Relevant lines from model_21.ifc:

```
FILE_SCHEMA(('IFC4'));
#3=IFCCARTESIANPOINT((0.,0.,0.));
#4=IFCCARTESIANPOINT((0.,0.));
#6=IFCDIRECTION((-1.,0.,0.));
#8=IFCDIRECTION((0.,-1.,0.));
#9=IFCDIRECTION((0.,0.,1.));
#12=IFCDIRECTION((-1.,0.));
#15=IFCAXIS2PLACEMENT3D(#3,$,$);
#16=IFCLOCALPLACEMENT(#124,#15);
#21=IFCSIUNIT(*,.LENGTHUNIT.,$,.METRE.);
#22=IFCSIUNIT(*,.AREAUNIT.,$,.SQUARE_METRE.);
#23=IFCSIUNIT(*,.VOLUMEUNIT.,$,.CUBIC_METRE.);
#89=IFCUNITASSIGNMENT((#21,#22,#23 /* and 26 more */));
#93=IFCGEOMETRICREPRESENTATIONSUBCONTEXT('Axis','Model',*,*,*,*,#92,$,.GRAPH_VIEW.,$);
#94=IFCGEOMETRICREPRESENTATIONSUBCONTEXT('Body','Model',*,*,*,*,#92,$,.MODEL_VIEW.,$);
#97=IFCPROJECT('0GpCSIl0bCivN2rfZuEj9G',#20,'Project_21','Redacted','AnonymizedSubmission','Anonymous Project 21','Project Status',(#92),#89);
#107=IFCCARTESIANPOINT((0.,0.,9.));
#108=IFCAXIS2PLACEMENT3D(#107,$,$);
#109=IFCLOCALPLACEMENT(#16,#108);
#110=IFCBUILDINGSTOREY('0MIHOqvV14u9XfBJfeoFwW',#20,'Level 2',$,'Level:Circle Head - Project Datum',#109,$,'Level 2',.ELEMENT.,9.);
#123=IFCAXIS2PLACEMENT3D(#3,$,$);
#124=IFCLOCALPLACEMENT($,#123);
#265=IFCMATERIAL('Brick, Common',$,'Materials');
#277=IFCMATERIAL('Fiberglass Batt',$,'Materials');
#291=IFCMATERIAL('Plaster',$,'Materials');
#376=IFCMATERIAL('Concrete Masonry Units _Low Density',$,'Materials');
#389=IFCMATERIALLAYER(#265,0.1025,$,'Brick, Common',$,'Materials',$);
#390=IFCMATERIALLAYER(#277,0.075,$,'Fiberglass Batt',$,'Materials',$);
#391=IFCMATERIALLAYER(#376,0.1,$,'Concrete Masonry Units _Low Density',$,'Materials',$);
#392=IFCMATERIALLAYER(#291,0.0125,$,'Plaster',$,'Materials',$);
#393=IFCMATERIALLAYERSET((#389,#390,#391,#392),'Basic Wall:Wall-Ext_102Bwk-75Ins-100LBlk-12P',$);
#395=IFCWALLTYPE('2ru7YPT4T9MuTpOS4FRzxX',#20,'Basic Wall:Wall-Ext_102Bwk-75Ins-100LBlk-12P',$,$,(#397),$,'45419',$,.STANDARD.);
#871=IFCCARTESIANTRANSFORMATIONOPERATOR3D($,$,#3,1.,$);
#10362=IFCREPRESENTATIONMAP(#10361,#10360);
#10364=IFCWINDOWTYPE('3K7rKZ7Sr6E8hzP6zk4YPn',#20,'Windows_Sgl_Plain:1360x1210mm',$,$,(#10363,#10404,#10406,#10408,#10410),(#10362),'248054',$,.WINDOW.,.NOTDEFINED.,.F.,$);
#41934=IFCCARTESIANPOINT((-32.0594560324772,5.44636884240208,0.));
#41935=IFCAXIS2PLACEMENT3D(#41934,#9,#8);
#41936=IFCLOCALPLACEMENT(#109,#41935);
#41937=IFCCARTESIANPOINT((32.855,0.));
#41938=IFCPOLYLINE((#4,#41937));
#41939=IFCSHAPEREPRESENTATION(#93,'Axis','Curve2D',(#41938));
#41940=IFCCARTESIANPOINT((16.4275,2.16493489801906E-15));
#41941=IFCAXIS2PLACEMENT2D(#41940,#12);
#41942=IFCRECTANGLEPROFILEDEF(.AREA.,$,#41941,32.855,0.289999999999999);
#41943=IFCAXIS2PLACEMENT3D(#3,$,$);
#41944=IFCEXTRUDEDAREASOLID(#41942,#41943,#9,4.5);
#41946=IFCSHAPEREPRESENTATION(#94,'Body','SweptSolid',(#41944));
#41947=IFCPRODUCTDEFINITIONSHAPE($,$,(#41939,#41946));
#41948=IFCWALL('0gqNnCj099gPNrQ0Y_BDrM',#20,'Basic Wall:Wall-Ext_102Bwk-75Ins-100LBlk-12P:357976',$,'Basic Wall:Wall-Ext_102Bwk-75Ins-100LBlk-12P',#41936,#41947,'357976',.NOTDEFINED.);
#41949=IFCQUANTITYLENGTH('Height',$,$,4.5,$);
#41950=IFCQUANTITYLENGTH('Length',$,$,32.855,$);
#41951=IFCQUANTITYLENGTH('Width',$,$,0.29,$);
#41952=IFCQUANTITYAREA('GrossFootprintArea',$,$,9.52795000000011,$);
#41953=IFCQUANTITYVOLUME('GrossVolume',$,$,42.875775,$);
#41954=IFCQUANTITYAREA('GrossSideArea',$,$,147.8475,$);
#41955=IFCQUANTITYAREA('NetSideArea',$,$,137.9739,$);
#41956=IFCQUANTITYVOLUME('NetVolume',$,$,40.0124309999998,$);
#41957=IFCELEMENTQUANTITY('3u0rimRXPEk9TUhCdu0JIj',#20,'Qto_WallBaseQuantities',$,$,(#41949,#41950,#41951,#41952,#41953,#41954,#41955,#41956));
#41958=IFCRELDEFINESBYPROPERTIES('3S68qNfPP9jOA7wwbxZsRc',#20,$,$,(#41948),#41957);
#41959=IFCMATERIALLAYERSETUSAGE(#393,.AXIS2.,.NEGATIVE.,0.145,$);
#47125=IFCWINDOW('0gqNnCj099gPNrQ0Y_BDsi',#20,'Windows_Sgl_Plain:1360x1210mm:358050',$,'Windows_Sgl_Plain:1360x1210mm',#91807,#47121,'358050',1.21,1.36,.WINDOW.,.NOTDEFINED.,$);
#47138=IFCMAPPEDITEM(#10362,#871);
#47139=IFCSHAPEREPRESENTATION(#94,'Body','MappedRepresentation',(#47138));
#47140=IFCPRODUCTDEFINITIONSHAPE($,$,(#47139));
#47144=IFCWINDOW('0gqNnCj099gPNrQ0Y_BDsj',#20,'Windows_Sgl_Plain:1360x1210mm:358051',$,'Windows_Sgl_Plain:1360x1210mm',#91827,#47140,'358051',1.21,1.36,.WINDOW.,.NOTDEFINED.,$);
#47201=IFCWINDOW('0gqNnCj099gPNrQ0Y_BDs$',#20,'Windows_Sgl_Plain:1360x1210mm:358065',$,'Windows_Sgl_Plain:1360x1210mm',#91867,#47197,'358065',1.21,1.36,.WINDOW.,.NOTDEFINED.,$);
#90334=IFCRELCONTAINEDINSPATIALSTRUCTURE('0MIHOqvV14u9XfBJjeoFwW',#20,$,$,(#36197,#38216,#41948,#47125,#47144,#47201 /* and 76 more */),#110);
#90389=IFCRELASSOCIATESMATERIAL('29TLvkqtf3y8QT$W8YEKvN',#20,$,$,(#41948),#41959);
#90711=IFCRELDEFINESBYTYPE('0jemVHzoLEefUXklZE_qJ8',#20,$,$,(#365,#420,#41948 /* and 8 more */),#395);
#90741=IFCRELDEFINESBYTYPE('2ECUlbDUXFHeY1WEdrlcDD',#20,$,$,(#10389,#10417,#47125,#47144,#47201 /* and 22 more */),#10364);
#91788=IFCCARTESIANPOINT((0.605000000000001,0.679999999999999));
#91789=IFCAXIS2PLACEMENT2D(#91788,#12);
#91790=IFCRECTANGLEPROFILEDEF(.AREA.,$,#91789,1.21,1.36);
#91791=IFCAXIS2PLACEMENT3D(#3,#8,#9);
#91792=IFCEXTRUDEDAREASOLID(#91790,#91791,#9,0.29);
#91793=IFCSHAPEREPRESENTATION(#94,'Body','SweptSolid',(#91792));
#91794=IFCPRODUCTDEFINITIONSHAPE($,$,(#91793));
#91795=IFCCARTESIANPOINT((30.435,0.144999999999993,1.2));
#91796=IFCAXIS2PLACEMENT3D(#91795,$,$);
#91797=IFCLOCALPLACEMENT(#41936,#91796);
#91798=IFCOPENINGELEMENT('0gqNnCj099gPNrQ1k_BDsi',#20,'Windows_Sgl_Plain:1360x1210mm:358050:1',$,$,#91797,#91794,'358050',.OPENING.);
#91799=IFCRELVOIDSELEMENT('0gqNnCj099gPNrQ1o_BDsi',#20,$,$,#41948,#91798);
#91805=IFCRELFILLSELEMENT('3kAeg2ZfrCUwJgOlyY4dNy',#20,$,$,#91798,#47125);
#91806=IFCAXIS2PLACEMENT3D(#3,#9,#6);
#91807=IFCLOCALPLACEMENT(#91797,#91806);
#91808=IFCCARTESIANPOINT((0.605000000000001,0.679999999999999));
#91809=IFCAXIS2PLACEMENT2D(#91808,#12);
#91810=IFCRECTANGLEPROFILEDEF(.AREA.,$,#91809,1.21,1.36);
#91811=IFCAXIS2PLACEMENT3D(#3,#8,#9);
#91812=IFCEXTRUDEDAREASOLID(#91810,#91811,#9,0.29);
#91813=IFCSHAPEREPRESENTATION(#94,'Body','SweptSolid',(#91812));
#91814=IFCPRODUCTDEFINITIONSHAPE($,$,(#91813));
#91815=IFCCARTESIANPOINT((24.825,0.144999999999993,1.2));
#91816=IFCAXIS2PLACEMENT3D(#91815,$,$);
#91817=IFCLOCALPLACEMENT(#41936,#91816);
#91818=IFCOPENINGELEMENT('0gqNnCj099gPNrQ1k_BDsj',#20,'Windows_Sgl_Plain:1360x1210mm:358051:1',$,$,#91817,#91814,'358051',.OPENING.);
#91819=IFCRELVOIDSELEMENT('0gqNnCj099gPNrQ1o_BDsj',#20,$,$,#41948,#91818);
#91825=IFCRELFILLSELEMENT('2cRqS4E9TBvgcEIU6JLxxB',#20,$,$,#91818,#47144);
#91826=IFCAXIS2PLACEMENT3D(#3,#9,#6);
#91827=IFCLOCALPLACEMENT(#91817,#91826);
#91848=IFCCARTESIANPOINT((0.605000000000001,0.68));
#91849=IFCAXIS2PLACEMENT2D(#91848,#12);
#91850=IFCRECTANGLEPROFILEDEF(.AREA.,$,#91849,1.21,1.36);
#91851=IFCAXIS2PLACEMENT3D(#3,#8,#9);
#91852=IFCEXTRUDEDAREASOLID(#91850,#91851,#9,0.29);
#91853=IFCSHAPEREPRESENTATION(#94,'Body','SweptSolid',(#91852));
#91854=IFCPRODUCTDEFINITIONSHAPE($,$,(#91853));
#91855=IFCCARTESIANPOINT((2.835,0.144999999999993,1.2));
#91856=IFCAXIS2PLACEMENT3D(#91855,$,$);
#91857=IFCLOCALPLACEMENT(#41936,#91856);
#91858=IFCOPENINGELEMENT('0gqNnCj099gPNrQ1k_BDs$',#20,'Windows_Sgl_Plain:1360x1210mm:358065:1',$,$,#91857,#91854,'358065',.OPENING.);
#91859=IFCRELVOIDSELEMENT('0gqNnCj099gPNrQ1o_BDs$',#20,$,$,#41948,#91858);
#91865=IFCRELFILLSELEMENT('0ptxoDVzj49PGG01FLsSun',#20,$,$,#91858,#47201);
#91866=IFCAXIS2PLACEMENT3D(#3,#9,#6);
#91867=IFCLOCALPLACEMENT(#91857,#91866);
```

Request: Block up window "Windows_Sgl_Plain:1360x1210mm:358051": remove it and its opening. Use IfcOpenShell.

```python
import ifcopenshell
import ifcopenshell.api.feature
import ifcopenshell.api.pset
import ifcopenshell.api.root
import ifcopenshell.geom
import ifcopenshell.util.element
import ifcopenshell.util.shape
import ifcopenshell.util.unit

model = ifcopenshell.open("model_21.ifc")
area_scale = ifcopenshell.util.unit.calculate_unit_scale(model, "AREAUNIT")
volume_scale = ifcopenshell.util.unit.calculate_unit_scale(model, "VOLUMEUNIT")
settings = ifcopenshell.geom.settings()


def volume(element):
    """Net volume in cubic metres, openings subtracted."""
    shape = ifcopenshell.geom.create_shape(settings, element)
    return ifcopenshell.util.shape.get_volume(shape.geometry)


window = model.by_guid("0gqNnCj099gPNrQ0Y_BDsj")
opening = window.FillsVoids[0].RelatingOpeningElement
wall = opening.VoidsElements[0].RelatingBuildingElement
before = volume(wall)

ifcopenshell.api.root.remove_product(model, product=window)
ifcopenshell.api.feature.remove_feature(model, feature=opening)

after = volume(wall)
thickness = 0.29  # wall thickness in metres

# Update the wall's stored quantities.
qto = model.by_id(ifcopenshell.util.element.get_pset(wall, "Qto_WallBaseQuantities", should_inherit=False)["id"])
ifcopenshell.api.pset.edit_qto(model, qto=qto, properties={
    "NetSideArea": after / thickness / area_scale,
    "NetVolume": after / volume_scale,
})

print(f"wall volume {before:.3f} -> {after:.3f} m3")

model.write("model_21_rev.ifc")
```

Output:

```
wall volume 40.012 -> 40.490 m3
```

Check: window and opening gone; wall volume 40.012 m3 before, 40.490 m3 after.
